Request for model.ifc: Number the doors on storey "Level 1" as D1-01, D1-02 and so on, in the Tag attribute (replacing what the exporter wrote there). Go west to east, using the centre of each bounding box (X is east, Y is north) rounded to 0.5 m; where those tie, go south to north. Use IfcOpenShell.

First a look at what the model holds.

```python
import ifcopenshell
import ifcopenshell.util.element
import ifcopenshell.util.placement

model = ifcopenshell.open("model.ifc")
print(model.schema)
storey = next(s for s in model.by_type("IfcBuildingStorey") if s.Name == "Level 1")
doors = [e for e in ifcopenshell.util.element.get_decomposition(storey) if e.is_a("IfcDoor")]
for e in sorted(doors, key=lambda e: e.id()):
    origin = ifcopenshell.util.placement.get_local_placement(e.ObjectPlacement)[:3, 3]
    print(e.id(), e.Tag, e.Name, origin.round(2) + 0.0, sep=" | ")
```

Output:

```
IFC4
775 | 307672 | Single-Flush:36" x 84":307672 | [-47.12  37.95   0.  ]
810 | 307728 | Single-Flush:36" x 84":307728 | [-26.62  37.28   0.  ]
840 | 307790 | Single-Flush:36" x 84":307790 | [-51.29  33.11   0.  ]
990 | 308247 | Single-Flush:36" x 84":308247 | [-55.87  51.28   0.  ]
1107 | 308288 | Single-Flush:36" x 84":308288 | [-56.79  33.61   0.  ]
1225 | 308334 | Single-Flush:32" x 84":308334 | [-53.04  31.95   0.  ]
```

```python
import ifcopenshell
import ifcopenshell.geom
import ifcopenshell.util.element
import ifcopenshell.util.shape

model = ifcopenshell.open("model.ifc")
settings = ifcopenshell.geom.settings()
settings.set("use-world-coords", True)


def centre(element):
    shape = ifcopenshell.geom.create_shape(settings, element)
    return ifcopenshell.util.shape.get_bbox_centroid(shape.geometry)


storey = next(s for s in model.by_type("IfcBuildingStorey") if s.Name == "Level 1")
doors = [e for e in ifcopenshell.util.element.get_decomposition(storey) if e.is_a("IfcDoor")]

# Insertion points can sit at a corner or the storey origin, so sort by the geometry (in metres).
centres = {e: centre(e) for e in doors}
doors.sort(key=lambda e: (round(centres[e][0] / 0.5), centres[e][1]))

for i, e in enumerate(doors, start=1):
    number = f"D1-{i:02d}"
    e.Tag = number
    print(e.id(), number)

model.write("model-out.ifc")
```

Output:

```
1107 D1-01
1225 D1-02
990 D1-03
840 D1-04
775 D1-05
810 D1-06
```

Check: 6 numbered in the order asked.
